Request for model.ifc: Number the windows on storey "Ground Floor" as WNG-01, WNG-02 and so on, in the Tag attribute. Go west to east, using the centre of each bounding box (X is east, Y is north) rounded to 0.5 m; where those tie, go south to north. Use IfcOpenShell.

First a look at what the model holds.

```python
import ifcopenshell
import ifcopenshell.util.element
import ifcopenshell.util.placement

model = ifcopenshell.open("model.ifc")
print(model.schema)
storey = next(s for s in model.by_type("IfcBuildingStorey") if s.Name == "Ground Floor")
windows = [e for e in ifcopenshell.util.element.get_decomposition(storey) if e.is_a("IfcWindow")]
for e in sorted(windows, key=lambda e: e.id()):
    origin = ifcopenshell.util.placement.get_local_placement(e.ObjectPlacement)[:3, 3]
    print(e.id(), e.Tag, e.Name, origin.round(2) + 0.0, sep=" | ")
```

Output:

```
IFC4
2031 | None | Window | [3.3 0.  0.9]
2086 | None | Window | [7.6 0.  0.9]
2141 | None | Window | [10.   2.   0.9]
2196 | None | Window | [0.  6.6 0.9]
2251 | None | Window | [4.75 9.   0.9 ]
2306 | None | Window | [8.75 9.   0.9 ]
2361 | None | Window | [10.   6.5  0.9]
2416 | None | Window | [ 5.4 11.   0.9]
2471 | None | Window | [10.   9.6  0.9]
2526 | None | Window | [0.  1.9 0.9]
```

```python
import ifcopenshell
import ifcopenshell.geom
import ifcopenshell.util.element
import ifcopenshell.util.shape

model = ifcopenshell.open("model.ifc")
settings = ifcopenshell.geom.settings()
settings.set("use-world-coords", True)


def centre(element):
    shape = ifcopenshell.geom.create_shape(settings, element)
    return ifcopenshell.util.shape.get_bbox_centroid(shape.geometry)


storey = next(s for s in model.by_type("IfcBuildingStorey") if s.Name == "Ground Floor")
windows = [e for e in ifcopenshell.util.element.get_decomposition(storey) if e.is_a("IfcWindow")]

# Insertion points can sit at a corner or the storey origin, so sort by the geometry (in metres).
centres = {e: centre(e) for e in windows}
windows.sort(key=lambda e: (round(centres[e][0] / 0.5), centres[e][1]))

for i, e in enumerate(windows, start=1):
    number = f"WNG-{i:02d}"
    e.Tag = number
    print(e.id(), number)

model.write("model-out.ifc")
```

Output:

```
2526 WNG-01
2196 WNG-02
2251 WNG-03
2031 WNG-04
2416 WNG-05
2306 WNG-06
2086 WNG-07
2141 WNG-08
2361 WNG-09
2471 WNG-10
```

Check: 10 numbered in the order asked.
